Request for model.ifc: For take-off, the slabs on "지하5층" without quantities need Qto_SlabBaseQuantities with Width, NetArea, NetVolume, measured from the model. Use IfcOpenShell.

First a look at what the model holds.

```python
import ifcopenshell
import ifcopenshell.util.element
import ifcopenshell.util.unit

model = ifcopenshell.open("model.ifc")
print(model.schema)
for unit_type in ("LENGTHUNIT", "AREAUNIT", "VOLUMEUNIT"):
    print(unit_type, ifcopenshell.util.unit.calculate_unit_scale(model, unit_type))
storey = next(s for s in model.by_type("IfcBuildingStorey") if s.Name == "지하5층")
slabs = [e for e in ifcopenshell.util.element.get_decomposition(storey) if e.is_a("IfcSlab")]
for e in sorted(slabs, key=lambda e: e.id()):
    print(e.id(), e.is_a(), e.Name, list(ifcopenshell.util.element.get_psets(e, qtos_only=True)), sep=" | ")
```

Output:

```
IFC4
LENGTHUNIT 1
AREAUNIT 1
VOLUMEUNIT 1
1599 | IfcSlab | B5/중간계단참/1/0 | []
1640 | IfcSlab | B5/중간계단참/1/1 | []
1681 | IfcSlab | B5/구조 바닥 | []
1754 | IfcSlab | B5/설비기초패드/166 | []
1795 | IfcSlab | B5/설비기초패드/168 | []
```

```python
import ifcopenshell
import ifcopenshell.api.pset
import ifcopenshell.geom
import ifcopenshell.util.element
import ifcopenshell.util.shape
import ifcopenshell.util.unit

model = ifcopenshell.open("model.ifc")
unit_scale = ifcopenshell.util.unit.calculate_unit_scale(model)
area_scale = ifcopenshell.util.unit.calculate_unit_scale(model, "AREAUNIT")
volume_scale = ifcopenshell.util.unit.calculate_unit_scale(model, "VOLUMEUNIT")
settings = ifcopenshell.geom.settings()

storey = next(s for s in model.by_type("IfcBuildingStorey") if s.Name == "지하5층")
slabs = [e for e in ifcopenshell.util.element.get_decomposition(storey) if e.is_a("IfcSlab")]

for e in sorted(slabs, key=lambda e: e.id()):
    if ifcopenshell.util.element.get_psets(e, qtos_only=True, should_inherit=False):
        continue
    # Geometry comes back in metres, in the element's own axes.
    shape = ifcopenshell.geom.create_shape(settings, e)
    values = {
        "Width": ifcopenshell.util.shape.get_z(shape.geometry) / unit_scale,
        "NetArea": ifcopenshell.util.shape.get_footprint_area(shape.geometry) / area_scale,
        "NetVolume": ifcopenshell.util.shape.get_volume(shape.geometry) / volume_scale,
    }
    qto = ifcopenshell.api.pset.add_qto(model, product=e, name="Qto_SlabBaseQuantities")
    ifcopenshell.api.pset.edit_qto(model, qto=qto, properties=values)
    print(e.id(), {k: round(v, 3) for k, v in values.items()})

model.write("model-out.ifc")
```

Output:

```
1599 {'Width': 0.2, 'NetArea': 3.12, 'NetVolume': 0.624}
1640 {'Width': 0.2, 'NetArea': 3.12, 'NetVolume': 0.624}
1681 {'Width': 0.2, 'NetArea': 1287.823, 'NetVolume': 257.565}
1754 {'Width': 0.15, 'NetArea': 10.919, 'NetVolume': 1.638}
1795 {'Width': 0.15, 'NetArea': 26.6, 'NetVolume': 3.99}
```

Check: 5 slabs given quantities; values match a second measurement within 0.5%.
